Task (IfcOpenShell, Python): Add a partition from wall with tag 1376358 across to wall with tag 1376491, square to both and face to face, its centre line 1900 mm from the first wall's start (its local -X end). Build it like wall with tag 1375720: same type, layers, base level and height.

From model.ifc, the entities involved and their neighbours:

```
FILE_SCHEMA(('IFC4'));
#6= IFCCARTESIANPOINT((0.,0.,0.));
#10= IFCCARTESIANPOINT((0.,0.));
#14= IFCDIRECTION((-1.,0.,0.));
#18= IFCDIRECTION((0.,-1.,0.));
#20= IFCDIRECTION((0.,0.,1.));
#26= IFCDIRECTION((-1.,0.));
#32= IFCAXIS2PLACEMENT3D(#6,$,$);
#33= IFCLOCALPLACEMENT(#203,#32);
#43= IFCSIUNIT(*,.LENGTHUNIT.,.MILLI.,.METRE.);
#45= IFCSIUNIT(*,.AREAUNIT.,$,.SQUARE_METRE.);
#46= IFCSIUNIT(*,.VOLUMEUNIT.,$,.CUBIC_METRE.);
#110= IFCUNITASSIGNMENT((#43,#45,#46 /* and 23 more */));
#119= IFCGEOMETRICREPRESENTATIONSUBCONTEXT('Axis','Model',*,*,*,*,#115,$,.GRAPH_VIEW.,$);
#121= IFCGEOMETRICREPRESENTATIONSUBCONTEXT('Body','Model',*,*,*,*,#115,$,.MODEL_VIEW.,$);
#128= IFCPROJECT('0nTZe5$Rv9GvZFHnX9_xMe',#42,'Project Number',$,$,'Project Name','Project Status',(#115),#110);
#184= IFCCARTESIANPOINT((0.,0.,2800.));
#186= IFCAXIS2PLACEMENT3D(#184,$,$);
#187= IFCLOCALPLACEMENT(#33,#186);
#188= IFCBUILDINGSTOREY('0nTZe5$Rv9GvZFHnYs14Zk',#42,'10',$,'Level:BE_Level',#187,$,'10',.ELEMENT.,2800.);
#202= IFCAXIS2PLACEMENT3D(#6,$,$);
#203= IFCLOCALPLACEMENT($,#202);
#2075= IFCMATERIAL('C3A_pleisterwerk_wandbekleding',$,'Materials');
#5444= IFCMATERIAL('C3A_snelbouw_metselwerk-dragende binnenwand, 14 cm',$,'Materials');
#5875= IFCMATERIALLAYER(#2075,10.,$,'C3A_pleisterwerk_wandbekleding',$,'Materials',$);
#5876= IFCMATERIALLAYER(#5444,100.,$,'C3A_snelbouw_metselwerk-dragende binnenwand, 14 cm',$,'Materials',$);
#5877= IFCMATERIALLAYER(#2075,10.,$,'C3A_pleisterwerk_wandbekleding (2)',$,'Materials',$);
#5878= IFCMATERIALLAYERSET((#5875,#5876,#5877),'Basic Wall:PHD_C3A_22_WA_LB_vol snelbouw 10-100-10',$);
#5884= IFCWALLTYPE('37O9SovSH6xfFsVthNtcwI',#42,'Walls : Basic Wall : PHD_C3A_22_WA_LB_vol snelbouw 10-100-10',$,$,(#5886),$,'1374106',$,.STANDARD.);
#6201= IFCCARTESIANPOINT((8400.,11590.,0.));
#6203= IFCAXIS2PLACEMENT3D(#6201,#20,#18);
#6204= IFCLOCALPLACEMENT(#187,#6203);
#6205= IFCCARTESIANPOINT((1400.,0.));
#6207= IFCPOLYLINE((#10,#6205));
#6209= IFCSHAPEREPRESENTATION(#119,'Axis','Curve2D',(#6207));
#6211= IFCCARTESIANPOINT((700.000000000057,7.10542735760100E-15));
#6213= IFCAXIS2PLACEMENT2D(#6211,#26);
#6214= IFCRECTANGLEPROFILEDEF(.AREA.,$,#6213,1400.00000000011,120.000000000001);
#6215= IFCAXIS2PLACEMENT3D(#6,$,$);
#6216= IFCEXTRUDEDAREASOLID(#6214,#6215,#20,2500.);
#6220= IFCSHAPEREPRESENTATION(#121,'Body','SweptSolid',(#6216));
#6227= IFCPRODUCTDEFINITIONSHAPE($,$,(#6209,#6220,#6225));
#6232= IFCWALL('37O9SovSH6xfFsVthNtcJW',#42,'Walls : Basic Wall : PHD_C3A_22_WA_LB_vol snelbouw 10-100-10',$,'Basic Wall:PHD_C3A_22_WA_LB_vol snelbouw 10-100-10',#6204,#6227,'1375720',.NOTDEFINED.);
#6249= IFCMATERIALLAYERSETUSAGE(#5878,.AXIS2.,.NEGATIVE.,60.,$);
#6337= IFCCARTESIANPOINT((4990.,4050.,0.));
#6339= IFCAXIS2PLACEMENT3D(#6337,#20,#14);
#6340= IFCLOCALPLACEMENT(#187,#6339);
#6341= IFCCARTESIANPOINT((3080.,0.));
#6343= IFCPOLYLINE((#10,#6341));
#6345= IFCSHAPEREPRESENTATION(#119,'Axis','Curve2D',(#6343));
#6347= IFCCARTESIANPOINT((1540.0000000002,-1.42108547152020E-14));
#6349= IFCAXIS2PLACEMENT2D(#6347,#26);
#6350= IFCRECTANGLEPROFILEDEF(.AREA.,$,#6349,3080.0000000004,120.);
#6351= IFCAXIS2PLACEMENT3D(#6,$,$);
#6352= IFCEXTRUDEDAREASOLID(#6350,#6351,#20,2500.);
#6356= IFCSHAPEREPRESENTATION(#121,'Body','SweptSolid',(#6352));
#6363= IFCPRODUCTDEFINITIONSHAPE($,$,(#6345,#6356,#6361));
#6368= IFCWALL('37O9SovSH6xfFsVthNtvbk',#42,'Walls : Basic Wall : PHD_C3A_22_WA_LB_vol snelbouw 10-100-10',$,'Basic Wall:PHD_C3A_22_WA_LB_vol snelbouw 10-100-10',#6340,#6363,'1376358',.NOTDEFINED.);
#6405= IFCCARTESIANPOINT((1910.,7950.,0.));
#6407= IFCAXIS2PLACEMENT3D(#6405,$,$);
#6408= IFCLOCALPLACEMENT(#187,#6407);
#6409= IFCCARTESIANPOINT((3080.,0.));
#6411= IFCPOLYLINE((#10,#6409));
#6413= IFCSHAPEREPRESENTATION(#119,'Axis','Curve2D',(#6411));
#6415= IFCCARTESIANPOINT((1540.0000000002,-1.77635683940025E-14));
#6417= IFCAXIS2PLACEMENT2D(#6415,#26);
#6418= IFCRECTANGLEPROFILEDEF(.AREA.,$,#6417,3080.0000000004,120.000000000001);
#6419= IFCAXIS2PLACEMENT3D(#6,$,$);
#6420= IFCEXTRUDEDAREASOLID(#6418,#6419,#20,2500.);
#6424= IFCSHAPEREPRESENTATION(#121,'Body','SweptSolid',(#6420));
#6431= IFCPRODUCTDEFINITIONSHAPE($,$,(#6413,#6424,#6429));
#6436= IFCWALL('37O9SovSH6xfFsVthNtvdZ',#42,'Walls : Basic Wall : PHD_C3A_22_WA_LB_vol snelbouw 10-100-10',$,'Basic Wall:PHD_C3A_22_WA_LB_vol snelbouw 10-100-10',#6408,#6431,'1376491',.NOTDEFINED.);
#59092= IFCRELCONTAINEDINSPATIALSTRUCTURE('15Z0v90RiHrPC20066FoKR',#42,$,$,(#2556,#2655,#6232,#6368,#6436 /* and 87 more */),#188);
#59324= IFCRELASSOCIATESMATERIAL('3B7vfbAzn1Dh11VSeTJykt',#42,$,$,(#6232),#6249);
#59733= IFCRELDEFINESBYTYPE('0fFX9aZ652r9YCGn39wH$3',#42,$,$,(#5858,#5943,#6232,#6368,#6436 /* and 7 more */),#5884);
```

```python
import numpy as np
import ifcopenshell
import ifcopenshell.api.geometry
import ifcopenshell.api.material
import ifcopenshell.api.pset
import ifcopenshell.api.root
import ifcopenshell.api.spatial
import ifcopenshell.api.type
import ifcopenshell.geom
import ifcopenshell.util.element
import ifcopenshell.util.placement
import ifcopenshell.util.representation
import ifcopenshell.util.shape
import ifcopenshell.util.unit

model = ifcopenshell.open("model.ifc")
unit_scale = ifcopenshell.util.unit.calculate_unit_scale(model)
settings = ifcopenshell.geom.settings()
settings.set("use-world-coords", True)

start_wall = model.by_guid("37O9SovSH6xfFsVthNtvbk")
end_wall = model.by_id(6436)
like = model.by_guid("37O9SovSH6xfFsVthNtcJW")
matrix = ifcopenshell.util.placement.get_local_placement(start_wall.ObjectPlacement)
matrix[:3, 3] *= unit_scale


def extent(element):
    """Bounding box in the first wall's axes, in metres."""
    shape = ifcopenshell.geom.create_shape(settings, element)
    points = (ifcopenshell.util.shape.get_vertices(shape.geometry) - matrix[:3, 3]) @ matrix[:3, :3]
    return points.min(axis=0), points.max(axis=0)


y_start = extent(start_wall)[0][1]
y_end = extent(end_wall)[1][1]
like_min, like_max = extent(like)
length, height = float(abs(y_end - y_start)), float(like_max[2] - like_min[2])
layer_set = ifcopenshell.util.element.get_material(like, should_skip_usage=True)
thickness = sum(layer.LayerThickness for layer in layer_set.MaterialLayers) * unit_scale

wall = ifcopenshell.api.root.create_entity(model, ifc_class="IfcWall", name="New partition")
storey = ifcopenshell.util.element.get_container(like)
ifcopenshell.api.spatial.assign_container(model, products=[wall], relating_structure=storey)
ifcopenshell.api.type.assign_type(
    model, related_objects=[wall], relating_type=ifcopenshell.util.element.get_type(like), should_map_representations=False
)
rel = ifcopenshell.api.material.assign_material(
    model, products=[wall], type="IfcMaterialLayerSetUsage", material=layer_set
)
rel.RelatingMaterial.OffsetFromReferenceLine = -thickness / 2 / unit_scale
pset = ifcopenshell.api.pset.add_pset(model, product=wall, name="Pset_WallCommon")
ifcopenshell.api.pset.edit_pset(model, pset=pset, properties={"IsExternal": False, "LoadBearing": False})

# The axis runs down the middle of the wall.
axis = ifcopenshell.api.geometry.add_axis_representation(
    model, context=ifcopenshell.util.representation.get_context(model, "Model", "Axis"), axis=[(0.0, 0.0), (length, 0.0)]
)
body = ifcopenshell.api.geometry.add_wall_representation(
    model,
    context=ifcopenshell.util.representation.get_context(model, "Model", "Body", "MODEL_VIEW"),
    length=length,
    height=height,
    thickness=thickness,
    offset=-thickness / 2,
)
for representation in (axis, body):
    ifcopenshell.api.geometry.assign_representation(model, product=wall, representation=representation)

placement = matrix @ ifcopenshell.util.placement.rotation(-90, "Z")
placement[:, 3] = matrix @ np.array([extent(start_wall)[0][0] + 1.9, y_start, like_min[2], 1.0])
ifcopenshell.api.geometry.edit_object_placement(model, product=wall, matrix=placement)

print(f"partition {length:.3f} m long, {height:.3f} m high, {thickness:.3f} m thick")

model.write("model_rev.ifc")
```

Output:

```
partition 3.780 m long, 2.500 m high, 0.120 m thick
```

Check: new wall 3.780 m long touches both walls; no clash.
